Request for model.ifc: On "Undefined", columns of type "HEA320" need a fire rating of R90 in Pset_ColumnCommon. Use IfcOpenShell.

First a look at what the model holds.

```python
import ifcopenshell
import ifcopenshell.util.element

model = ifcopenshell.open("model.ifc")
print(model.schema)
storey = next(s for s in model.by_type("IfcBuildingStorey") if s.Name == "Undefined")
columns = [e for e in ifcopenshell.util.element.get_decomposition(storey) if e.is_a("IfcColumn")]
seen = {}
for e in columns:
    element_type = ifcopenshell.util.element.get_type(e)
    key = (element_type.Name if element_type != e and element_type else None, ifcopenshell.util.element.get_pset(e, "Pset_ColumnCommon", "FireRating"))
    seen[key] = seen.get(key, 0) + 1
for (name, value), count in sorted(seen.items(), key=str):
    print(count, "x", name, "|", value)
```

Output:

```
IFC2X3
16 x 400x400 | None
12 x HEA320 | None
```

```python
import ifcopenshell
import ifcopenshell.api.pset
import ifcopenshell.util.element

model = ifcopenshell.open("model.ifc")

storey = next(s for s in model.by_type("IfcBuildingStorey") if s.Name == "Undefined")
columns = [e for e in ifcopenshell.util.element.get_decomposition(storey) if e.is_a("IfcColumn")]

count = 0
for e in columns:
    element_type = ifcopenshell.util.element.get_type(e)
    if element_type in (None, e) or element_type.Name != "HEA320":
        continue
    found = ifcopenshell.util.element.get_pset(e, "Pset_ColumnCommon", should_inherit=False)
    if found:
        pset = model.by_id(found["id"])
        if len(ifcopenshell.util.element.get_elements_by_pset(pset)) > 1:
            pset = ifcopenshell.api.pset.unshare_pset(model, products=[e], pset=pset)[0]
    else:
        pset = ifcopenshell.api.pset.add_pset(model, product=e, name="Pset_ColumnCommon")
    ifcopenshell.api.pset.edit_pset(model, pset=pset, properties={"FireRating": "R90"})
    count += 1

print(count, "columns updated")

model.write("model-out.ifc")
```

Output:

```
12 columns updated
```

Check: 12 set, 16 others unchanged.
